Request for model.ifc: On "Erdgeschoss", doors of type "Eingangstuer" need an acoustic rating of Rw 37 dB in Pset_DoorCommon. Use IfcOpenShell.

First a look at what the model holds.

```python
import ifcopenshell
import ifcopenshell.util.element

model = ifcopenshell.open("model.ifc")
print(model.schema)
storey = next(s for s in model.by_type("IfcBuildingStorey") if s.Name == "Erdgeschoss")
doors = [e for e in ifcopenshell.util.element.get_decomposition(storey) if e.is_a("IfcDoor")]
seen = {}
for e in doors:
    element_type = ifcopenshell.util.element.get_type(e)
    key = (element_type.Name if element_type != e and element_type else None, ifcopenshell.util.element.get_pset(e, "Pset_DoorCommon", "AcousticRating"))
    seen[key] = seen.get(key, 0) + 1
for (name, value), count in sorted(seen.items(), key=str):
    print(count, "x", name, "|", value)
```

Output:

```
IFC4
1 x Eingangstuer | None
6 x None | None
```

```python
import ifcopenshell
import ifcopenshell.api.pset
import ifcopenshell.util.element

model = ifcopenshell.open("model.ifc")

storey = next(s for s in model.by_type("IfcBuildingStorey") if s.Name == "Erdgeschoss")
doors = [e for e in ifcopenshell.util.element.get_decomposition(storey) if e.is_a("IfcDoor")]

count = 0
for e in doors:
    element_type = ifcopenshell.util.element.get_type(e)
    if element_type in (None, e) or element_type.Name != "Eingangstuer":
        continue
    # add_pset returns the element's existing set when there is one.
    pset = ifcopenshell.api.pset.add_pset(model, product=e, name="Pset_DoorCommon")
    ifcopenshell.api.pset.edit_pset(model, pset=pset, properties={"AcousticRating": "Rw 37 dB"})
    count += 1

print(count, "doors updated")

model.write("model_edited.ifc")
```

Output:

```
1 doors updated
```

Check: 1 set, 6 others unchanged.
